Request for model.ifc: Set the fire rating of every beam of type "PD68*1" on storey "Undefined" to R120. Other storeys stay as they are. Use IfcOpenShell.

First a look at what the model holds.

```python
import ifcopenshell
import ifcopenshell.util.element

model = ifcopenshell.open("model.ifc")
print(model.schema)
storey = next(s for s in model.by_type("IfcBuildingStorey") if s.Name == "Undefined")
beams = [e for e in ifcopenshell.util.element.get_decomposition(storey) if e.is_a("IfcBeam")]
seen = {}
for e in beams:
    element_type = ifcopenshell.util.element.get_type(e)
    key = (element_type.Name if element_type != e and element_type else None, ifcopenshell.util.element.get_pset(e, "Pset_BeamCommon", "FireRating"))
    seen[key] = seen.get(key, 0) + 1
for (name, value), count in sorted(seen.items(), key=str):
    print(count, "x", name, "|", value)
```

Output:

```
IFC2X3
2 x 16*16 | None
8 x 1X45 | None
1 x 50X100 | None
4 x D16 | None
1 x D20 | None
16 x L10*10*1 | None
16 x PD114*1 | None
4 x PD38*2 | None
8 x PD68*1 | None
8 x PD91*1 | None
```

```python
import ifcopenshell
import ifcopenshell.api.pset
import ifcopenshell.util.element

model = ifcopenshell.open("model.ifc")

storey = next(s for s in model.by_type("IfcBuildingStorey") if s.Name == "Undefined")
beams = [e for e in ifcopenshell.util.element.get_decomposition(storey) if e.is_a("IfcBeam")]

count = 0
for e in beams:
    element_type = ifcopenshell.util.element.get_type(e)
    if element_type in (None, e) or element_type.Name != "PD68*1":
        continue
    # add_pset returns the element's existing set when there is one.
    pset = ifcopenshell.api.pset.add_pset(model, product=e, name="Pset_BeamCommon")
    ifcopenshell.api.pset.edit_pset(model, pset=pset, properties={"FireRating": "R120"})
    count += 1

print(count, "beams updated")

model.write("model-out.ifc")
```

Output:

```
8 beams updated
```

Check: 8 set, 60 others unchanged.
